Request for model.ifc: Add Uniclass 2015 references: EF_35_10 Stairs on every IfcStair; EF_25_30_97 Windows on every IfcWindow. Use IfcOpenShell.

First a look at what the model holds.

```python
import ifcopenshell

model = ifcopenshell.open("model.ifc")
print(model.schema)
print("classifications:", [c.Name for c in model.by_type("IfcClassification")])
for ifc_class in ("IfcDoor", "IfcRoof", "IfcStair", "IfcWall", "IfcWindow"):
    print(ifc_class, len(model.by_type(ifc_class)))
```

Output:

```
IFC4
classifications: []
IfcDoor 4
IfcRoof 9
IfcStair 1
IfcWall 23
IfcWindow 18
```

```python
import ifcopenshell
import ifcopenshell.api.classification

model = ifcopenshell.open("model.ifc")

system = ifcopenshell.api.classification.add_classification(model, classification="Uniclass 2015")

codes = {
    "IfcStair": ("EF_35_10", "Stairs"),
    "IfcWindow": ("EF_25_30_97", "Windows"),
}
for ifc_class, (code, name) in codes.items():
    products = model.by_type(ifc_class)
    ifcopenshell.api.classification.add_reference(
        model, products=products, classification=system, identification=code, name=name
    )
    print(code, len(products))

model.write("model-out.ifc")
```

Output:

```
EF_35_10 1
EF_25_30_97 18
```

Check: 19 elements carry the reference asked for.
